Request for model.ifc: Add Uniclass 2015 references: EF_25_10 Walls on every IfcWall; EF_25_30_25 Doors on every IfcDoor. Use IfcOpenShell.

First a look at what the model holds.

```python
import ifcopenshell

model = ifcopenshell.open("model.ifc")
print(model.schema)
print("classifications:", [c.Name for c in model.by_type("IfcClassification")])
for ifc_class in ("IfcDoor", "IfcRoof", "IfcStair", "IfcWall", "IfcWindow"):
    print(ifc_class, len(model.by_type(ifc_class)))
```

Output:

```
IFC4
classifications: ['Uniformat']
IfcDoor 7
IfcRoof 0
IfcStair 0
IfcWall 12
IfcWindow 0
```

```python
import ifcopenshell
import ifcopenshell.api.classification

model = ifcopenshell.open("model.ifc")

system = ifcopenshell.api.classification.add_classification(model, classification="Uniclass 2015")

codes = {
    "IfcWall": ("EF_25_10", "Walls"),
    "IfcDoor": ("EF_25_30_25", "Doors"),
}
for ifc_class, (code, name) in codes.items():
    products = model.by_type(ifc_class)
    ifcopenshell.api.classification.add_reference(
        model, products=products, classification=system, identification=code, name=name
    )
    print(code, len(products))

model.write("model_v2.ifc")
```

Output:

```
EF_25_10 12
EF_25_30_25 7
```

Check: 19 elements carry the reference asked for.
